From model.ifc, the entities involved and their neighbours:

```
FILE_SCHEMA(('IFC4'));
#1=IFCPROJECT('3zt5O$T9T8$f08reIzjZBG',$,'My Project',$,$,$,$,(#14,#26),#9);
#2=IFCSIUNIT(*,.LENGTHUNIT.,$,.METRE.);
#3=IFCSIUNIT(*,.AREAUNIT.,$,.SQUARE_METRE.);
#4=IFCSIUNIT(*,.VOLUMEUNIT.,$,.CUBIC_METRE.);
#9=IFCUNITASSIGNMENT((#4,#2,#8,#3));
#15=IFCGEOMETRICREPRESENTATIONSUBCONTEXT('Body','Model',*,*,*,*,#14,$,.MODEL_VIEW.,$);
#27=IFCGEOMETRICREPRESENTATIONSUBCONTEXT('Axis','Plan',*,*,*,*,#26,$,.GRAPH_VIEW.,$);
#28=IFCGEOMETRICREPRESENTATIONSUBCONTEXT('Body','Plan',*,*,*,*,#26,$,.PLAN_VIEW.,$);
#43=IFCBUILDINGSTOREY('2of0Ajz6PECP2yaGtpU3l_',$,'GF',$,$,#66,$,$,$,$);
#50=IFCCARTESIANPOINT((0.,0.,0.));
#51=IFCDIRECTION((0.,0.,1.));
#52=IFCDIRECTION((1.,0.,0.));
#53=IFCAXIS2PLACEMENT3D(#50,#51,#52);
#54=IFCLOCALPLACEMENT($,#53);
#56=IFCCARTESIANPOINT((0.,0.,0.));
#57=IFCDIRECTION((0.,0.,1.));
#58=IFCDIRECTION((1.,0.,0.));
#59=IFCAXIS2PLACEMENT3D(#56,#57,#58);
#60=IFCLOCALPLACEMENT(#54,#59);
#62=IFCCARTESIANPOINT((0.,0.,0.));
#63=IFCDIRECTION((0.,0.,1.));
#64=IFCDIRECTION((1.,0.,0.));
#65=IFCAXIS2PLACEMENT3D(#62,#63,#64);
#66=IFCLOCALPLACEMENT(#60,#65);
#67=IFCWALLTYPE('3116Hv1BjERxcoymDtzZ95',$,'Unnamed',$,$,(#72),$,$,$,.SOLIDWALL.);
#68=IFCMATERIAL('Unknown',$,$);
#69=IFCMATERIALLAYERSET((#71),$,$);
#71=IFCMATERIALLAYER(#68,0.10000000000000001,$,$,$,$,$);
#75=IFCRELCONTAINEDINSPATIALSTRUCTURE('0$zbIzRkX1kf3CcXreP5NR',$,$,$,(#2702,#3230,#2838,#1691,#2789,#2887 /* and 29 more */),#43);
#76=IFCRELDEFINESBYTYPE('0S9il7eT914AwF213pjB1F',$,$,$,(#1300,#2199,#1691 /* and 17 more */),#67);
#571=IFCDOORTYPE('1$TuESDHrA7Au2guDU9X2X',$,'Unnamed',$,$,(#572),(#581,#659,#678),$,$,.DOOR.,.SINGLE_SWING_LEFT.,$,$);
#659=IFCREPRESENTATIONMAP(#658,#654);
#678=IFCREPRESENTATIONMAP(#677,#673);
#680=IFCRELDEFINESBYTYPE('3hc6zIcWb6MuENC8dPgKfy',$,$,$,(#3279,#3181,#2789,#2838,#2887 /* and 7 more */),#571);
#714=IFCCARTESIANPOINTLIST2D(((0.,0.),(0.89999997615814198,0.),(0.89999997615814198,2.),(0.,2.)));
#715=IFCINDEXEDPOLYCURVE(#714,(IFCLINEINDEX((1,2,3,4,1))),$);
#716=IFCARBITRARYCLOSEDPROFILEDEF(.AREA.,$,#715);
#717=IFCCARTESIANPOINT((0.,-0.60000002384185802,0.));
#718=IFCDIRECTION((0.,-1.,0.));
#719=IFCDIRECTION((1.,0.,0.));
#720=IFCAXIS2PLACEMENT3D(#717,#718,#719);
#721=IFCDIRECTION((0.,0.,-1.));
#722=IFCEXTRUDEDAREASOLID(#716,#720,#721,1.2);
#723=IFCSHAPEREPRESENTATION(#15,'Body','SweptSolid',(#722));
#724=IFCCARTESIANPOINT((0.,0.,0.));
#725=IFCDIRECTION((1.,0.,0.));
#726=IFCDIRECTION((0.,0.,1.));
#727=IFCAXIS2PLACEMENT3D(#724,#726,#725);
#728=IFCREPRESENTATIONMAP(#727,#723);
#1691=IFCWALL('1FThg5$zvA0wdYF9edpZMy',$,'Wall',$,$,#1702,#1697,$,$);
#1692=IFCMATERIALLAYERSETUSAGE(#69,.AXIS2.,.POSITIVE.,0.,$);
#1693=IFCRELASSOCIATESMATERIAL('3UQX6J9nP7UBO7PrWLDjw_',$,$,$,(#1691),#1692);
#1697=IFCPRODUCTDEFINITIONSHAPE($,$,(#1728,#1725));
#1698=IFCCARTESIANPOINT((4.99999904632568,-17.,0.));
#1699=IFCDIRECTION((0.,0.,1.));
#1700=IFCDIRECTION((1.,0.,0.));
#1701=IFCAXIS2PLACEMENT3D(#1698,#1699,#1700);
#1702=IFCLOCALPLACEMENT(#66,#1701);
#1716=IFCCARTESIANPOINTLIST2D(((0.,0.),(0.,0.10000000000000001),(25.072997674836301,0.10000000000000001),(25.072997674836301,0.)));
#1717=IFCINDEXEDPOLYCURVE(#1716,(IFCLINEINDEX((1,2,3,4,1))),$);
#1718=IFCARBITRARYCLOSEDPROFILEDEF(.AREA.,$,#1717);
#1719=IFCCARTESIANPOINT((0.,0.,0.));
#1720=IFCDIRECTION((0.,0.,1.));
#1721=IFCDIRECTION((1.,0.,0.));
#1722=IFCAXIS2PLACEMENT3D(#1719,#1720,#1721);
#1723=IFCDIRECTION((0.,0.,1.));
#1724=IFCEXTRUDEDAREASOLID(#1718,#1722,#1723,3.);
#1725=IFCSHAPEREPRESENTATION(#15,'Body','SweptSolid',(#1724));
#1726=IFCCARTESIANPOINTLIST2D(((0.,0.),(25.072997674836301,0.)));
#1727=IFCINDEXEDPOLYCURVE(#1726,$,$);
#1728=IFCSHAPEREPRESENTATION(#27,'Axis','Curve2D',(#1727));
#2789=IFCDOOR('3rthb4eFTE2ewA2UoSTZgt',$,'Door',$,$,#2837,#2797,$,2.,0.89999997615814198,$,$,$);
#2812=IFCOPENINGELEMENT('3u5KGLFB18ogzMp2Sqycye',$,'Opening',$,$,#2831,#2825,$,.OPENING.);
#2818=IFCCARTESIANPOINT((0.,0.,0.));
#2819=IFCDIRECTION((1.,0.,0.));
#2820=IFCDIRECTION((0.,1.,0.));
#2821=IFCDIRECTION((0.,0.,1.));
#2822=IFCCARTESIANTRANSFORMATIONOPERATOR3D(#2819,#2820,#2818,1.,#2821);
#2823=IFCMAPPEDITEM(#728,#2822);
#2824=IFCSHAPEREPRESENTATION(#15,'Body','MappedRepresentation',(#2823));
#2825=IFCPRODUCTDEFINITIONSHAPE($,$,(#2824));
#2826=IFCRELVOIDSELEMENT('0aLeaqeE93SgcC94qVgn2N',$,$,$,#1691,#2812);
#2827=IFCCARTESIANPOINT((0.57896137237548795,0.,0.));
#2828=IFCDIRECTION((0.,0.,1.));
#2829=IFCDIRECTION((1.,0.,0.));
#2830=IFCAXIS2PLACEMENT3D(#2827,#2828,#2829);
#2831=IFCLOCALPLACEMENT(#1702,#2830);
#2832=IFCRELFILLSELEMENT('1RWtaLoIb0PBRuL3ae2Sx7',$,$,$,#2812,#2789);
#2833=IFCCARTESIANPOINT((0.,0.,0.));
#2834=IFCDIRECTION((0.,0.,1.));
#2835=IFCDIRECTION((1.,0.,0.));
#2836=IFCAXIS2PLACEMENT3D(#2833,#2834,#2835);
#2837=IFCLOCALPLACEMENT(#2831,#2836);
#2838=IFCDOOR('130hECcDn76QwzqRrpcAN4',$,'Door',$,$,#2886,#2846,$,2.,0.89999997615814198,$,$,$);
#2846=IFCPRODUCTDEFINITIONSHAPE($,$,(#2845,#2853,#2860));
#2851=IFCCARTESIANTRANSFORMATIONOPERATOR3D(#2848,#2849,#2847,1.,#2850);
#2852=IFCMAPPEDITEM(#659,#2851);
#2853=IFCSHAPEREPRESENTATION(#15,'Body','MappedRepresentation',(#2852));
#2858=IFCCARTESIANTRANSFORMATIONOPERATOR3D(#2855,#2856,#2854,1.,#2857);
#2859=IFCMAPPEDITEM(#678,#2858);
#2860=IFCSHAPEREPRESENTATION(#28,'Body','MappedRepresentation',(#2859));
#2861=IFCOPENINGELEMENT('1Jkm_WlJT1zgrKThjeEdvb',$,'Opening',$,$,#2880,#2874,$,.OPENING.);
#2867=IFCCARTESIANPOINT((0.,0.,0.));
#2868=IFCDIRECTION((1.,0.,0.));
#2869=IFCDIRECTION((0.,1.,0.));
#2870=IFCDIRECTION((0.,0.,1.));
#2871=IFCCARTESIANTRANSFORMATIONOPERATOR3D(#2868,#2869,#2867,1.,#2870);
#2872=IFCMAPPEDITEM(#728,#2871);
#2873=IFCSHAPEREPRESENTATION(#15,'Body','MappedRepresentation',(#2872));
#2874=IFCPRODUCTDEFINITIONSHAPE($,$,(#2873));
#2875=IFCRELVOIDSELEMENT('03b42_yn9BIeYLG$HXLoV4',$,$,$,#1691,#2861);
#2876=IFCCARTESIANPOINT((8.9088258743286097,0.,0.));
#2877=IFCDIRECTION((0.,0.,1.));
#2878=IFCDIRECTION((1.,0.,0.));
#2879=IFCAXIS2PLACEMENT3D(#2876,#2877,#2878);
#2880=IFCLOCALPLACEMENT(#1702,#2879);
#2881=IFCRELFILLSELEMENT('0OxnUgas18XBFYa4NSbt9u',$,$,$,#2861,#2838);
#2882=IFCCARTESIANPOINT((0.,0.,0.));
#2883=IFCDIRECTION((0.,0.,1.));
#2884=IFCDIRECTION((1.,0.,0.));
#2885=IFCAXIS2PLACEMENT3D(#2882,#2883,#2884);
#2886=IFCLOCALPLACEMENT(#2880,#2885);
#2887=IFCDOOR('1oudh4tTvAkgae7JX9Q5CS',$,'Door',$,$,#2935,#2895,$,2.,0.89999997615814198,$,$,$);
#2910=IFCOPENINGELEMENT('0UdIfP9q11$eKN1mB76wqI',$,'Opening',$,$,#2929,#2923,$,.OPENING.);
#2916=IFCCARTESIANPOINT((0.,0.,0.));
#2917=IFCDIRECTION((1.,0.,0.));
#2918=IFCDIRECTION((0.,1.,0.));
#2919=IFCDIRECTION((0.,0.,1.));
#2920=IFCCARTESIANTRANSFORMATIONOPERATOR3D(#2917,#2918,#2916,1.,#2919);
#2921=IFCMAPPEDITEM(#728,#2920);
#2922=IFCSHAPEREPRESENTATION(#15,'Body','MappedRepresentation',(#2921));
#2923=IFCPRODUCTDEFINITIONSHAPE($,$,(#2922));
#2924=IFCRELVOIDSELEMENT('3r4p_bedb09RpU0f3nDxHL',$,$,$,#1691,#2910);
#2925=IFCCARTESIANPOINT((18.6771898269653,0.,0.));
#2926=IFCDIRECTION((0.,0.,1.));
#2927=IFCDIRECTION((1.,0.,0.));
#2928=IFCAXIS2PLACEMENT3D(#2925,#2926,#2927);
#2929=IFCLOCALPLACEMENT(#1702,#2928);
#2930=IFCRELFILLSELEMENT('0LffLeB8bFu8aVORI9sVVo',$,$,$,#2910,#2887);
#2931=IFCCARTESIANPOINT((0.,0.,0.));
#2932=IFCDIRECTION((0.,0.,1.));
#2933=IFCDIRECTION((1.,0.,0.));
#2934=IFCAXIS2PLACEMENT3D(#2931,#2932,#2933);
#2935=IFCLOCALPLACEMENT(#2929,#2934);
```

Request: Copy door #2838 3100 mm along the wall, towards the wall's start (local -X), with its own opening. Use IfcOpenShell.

```python
import ifcopenshell
import ifcopenshell.api.feature
import ifcopenshell.api.geometry
import ifcopenshell.api.root
import ifcopenshell.geom
import ifcopenshell.util.element
import ifcopenshell.util.placement
import ifcopenshell.util.shape
import ifcopenshell.util.unit

model = ifcopenshell.open("model.ifc")
unit_scale = ifcopenshell.util.unit.calculate_unit_scale(model)
settings = ifcopenshell.geom.settings()


def volume(element):
    """Net volume in cubic metres, openings subtracted."""
    shape = ifcopenshell.geom.create_shape(settings, element)
    return ifcopenshell.util.shape.get_volume(shape.geometry)


door = model.by_guid("130hECcDn76QwzqRrpcAN4")
opening = door.FillsVoids[0].RelatingOpeningElement
wall = opening.VoidsElements[0].RelatingBuildingElement
before = volume(wall)
shift = ifcopenshell.util.placement.get_local_placement(wall.ObjectPlacement)[:3, 0] * -3.1 / unit_scale

# copy_class copies the void relationship, type, container and properties, but no geometry.
new_opening = ifcopenshell.api.root.copy_class(model, product=opening)
new_opening.Representation = ifcopenshell.util.element.copy_deep(
    model, opening.Representation, exclude=["IfcGeometricRepresentationContext", "IfcRepresentationMap"]
)
new_door = ifcopenshell.api.root.copy_class(model, product=door)
new_door.Representation = ifcopenshell.util.element.copy_deep(
    model, door.Representation, exclude=["IfcGeometricRepresentationContext", "IfcRepresentationMap"]
)
ifcopenshell.api.feature.add_filling(model, opening=new_opening, element=new_door)

for old, new in ((opening, new_opening), (door, new_door)):
    matrix = ifcopenshell.util.placement.get_local_placement(old.ObjectPlacement)
    matrix[:3, 3] += shift
    ifcopenshell.api.geometry.edit_object_placement(model, product=new, matrix=matrix, is_si=False)

after = volume(wall)

print(f"wall volume {before:.3f} -> {after:.3f} m3")

model.write("model-out.ifc")
```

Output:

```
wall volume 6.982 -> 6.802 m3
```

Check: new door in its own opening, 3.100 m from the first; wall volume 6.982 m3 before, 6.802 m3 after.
